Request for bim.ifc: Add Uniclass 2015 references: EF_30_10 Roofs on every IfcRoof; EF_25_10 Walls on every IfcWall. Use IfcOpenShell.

First a look at what the model holds.

```python
import ifcopenshell

model = ifcopenshell.open("bim.ifc")
print(model.schema)
print("classifications:", [c.Name for c in model.by_type("IfcClassification")])
for ifc_class in ("IfcDoor", "IfcRoof", "IfcStair", "IfcWall", "IfcWindow"):
    print(ifc_class, len(model.by_type(ifc_class)))
```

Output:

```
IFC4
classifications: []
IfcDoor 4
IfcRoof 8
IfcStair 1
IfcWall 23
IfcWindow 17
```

```python
import ifcopenshell
import ifcopenshell.api.classification

model = ifcopenshell.open("bim.ifc")

system = ifcopenshell.api.classification.add_classification(model, classification="Uniclass 2015")

codes = {
    "IfcRoof": ("EF_30_10", "Roofs"),
    "IfcWall": ("EF_25_10", "Walls"),
}
for ifc_class, (code, name) in codes.items():
    products = model.by_type(ifc_class)
    ifcopenshell.api.classification.add_reference(
        model, products=products, classification=system, identification=code, name=name
    )
    print(code, len(products))

model.write("bim_rev.ifc")
```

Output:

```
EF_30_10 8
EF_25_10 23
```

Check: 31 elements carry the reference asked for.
